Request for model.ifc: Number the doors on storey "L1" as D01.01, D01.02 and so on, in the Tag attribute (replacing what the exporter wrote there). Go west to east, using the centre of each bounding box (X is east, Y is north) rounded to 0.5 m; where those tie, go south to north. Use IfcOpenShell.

First a look at what the model holds.

```python
import ifcopenshell
import ifcopenshell.util.element
import ifcopenshell.util.placement

model = ifcopenshell.open("model.ifc")
print(model.schema)
storey = next(s for s in model.by_type("IfcBuildingStorey") if s.Name == "L1")
doors = [e for e in ifcopenshell.util.element.get_decomposition(storey) if e.is_a("IfcDoor")]
for e in sorted(doors, key=lambda e: e.id()):
    origin = ifcopenshell.util.placement.get_local_placement(e.ObjectPlacement)[:3, 3]
    print(e.id(), e.Tag, e.Name, origin.round(2) + 0.0, sep=" | ")
```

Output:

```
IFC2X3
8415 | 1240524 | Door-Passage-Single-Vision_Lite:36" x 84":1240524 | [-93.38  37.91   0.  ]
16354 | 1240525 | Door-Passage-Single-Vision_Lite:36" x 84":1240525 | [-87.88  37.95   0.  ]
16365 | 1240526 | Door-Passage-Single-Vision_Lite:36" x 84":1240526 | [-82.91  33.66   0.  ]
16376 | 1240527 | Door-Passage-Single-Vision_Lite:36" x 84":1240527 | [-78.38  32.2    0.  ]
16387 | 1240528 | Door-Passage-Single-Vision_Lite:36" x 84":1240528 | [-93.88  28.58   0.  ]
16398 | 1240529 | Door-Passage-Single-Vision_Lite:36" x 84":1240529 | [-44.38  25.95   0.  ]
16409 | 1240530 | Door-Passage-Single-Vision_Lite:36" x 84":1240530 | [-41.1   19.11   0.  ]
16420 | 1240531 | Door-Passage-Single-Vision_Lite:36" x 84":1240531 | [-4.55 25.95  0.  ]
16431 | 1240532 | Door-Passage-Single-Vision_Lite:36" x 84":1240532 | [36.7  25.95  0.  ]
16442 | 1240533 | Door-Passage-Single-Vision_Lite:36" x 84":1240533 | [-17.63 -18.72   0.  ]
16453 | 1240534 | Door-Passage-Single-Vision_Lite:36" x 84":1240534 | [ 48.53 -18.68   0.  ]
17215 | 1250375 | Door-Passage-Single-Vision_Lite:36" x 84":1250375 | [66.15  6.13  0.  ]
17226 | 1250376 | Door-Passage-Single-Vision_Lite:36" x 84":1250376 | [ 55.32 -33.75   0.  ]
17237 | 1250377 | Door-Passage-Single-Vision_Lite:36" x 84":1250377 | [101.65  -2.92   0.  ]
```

```python
import ifcopenshell
import ifcopenshell.geom
import ifcopenshell.util.element
import ifcopenshell.util.shape

model = ifcopenshell.open("model.ifc")
settings = ifcopenshell.geom.settings()
settings.set("use-world-coords", True)


def centre(element):
    shape = ifcopenshell.geom.create_shape(settings, element)
    return ifcopenshell.util.shape.get_bbox_centroid(shape.geometry)


storey = next(s for s in model.by_type("IfcBuildingStorey") if s.Name == "L1")
doors = [e for e in ifcopenshell.util.element.get_decomposition(storey) if e.is_a("IfcDoor")]

# Insertion points can sit at a corner or the storey origin, so sort by the geometry (in metres).
centres = {e: centre(e) for e in doors}
doors.sort(key=lambda e: (round(centres[e][0] / 0.5), centres[e][1]))

for i, e in enumerate(doors, start=1):
    number = f"D01.{i:02d}"
    e.Tag = number
    print(e.id(), number)

model.write("model_edited.ifc")
```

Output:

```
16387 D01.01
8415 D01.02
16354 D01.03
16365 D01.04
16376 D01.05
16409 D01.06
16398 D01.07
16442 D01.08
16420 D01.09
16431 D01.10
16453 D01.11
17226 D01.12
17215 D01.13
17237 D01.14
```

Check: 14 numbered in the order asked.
